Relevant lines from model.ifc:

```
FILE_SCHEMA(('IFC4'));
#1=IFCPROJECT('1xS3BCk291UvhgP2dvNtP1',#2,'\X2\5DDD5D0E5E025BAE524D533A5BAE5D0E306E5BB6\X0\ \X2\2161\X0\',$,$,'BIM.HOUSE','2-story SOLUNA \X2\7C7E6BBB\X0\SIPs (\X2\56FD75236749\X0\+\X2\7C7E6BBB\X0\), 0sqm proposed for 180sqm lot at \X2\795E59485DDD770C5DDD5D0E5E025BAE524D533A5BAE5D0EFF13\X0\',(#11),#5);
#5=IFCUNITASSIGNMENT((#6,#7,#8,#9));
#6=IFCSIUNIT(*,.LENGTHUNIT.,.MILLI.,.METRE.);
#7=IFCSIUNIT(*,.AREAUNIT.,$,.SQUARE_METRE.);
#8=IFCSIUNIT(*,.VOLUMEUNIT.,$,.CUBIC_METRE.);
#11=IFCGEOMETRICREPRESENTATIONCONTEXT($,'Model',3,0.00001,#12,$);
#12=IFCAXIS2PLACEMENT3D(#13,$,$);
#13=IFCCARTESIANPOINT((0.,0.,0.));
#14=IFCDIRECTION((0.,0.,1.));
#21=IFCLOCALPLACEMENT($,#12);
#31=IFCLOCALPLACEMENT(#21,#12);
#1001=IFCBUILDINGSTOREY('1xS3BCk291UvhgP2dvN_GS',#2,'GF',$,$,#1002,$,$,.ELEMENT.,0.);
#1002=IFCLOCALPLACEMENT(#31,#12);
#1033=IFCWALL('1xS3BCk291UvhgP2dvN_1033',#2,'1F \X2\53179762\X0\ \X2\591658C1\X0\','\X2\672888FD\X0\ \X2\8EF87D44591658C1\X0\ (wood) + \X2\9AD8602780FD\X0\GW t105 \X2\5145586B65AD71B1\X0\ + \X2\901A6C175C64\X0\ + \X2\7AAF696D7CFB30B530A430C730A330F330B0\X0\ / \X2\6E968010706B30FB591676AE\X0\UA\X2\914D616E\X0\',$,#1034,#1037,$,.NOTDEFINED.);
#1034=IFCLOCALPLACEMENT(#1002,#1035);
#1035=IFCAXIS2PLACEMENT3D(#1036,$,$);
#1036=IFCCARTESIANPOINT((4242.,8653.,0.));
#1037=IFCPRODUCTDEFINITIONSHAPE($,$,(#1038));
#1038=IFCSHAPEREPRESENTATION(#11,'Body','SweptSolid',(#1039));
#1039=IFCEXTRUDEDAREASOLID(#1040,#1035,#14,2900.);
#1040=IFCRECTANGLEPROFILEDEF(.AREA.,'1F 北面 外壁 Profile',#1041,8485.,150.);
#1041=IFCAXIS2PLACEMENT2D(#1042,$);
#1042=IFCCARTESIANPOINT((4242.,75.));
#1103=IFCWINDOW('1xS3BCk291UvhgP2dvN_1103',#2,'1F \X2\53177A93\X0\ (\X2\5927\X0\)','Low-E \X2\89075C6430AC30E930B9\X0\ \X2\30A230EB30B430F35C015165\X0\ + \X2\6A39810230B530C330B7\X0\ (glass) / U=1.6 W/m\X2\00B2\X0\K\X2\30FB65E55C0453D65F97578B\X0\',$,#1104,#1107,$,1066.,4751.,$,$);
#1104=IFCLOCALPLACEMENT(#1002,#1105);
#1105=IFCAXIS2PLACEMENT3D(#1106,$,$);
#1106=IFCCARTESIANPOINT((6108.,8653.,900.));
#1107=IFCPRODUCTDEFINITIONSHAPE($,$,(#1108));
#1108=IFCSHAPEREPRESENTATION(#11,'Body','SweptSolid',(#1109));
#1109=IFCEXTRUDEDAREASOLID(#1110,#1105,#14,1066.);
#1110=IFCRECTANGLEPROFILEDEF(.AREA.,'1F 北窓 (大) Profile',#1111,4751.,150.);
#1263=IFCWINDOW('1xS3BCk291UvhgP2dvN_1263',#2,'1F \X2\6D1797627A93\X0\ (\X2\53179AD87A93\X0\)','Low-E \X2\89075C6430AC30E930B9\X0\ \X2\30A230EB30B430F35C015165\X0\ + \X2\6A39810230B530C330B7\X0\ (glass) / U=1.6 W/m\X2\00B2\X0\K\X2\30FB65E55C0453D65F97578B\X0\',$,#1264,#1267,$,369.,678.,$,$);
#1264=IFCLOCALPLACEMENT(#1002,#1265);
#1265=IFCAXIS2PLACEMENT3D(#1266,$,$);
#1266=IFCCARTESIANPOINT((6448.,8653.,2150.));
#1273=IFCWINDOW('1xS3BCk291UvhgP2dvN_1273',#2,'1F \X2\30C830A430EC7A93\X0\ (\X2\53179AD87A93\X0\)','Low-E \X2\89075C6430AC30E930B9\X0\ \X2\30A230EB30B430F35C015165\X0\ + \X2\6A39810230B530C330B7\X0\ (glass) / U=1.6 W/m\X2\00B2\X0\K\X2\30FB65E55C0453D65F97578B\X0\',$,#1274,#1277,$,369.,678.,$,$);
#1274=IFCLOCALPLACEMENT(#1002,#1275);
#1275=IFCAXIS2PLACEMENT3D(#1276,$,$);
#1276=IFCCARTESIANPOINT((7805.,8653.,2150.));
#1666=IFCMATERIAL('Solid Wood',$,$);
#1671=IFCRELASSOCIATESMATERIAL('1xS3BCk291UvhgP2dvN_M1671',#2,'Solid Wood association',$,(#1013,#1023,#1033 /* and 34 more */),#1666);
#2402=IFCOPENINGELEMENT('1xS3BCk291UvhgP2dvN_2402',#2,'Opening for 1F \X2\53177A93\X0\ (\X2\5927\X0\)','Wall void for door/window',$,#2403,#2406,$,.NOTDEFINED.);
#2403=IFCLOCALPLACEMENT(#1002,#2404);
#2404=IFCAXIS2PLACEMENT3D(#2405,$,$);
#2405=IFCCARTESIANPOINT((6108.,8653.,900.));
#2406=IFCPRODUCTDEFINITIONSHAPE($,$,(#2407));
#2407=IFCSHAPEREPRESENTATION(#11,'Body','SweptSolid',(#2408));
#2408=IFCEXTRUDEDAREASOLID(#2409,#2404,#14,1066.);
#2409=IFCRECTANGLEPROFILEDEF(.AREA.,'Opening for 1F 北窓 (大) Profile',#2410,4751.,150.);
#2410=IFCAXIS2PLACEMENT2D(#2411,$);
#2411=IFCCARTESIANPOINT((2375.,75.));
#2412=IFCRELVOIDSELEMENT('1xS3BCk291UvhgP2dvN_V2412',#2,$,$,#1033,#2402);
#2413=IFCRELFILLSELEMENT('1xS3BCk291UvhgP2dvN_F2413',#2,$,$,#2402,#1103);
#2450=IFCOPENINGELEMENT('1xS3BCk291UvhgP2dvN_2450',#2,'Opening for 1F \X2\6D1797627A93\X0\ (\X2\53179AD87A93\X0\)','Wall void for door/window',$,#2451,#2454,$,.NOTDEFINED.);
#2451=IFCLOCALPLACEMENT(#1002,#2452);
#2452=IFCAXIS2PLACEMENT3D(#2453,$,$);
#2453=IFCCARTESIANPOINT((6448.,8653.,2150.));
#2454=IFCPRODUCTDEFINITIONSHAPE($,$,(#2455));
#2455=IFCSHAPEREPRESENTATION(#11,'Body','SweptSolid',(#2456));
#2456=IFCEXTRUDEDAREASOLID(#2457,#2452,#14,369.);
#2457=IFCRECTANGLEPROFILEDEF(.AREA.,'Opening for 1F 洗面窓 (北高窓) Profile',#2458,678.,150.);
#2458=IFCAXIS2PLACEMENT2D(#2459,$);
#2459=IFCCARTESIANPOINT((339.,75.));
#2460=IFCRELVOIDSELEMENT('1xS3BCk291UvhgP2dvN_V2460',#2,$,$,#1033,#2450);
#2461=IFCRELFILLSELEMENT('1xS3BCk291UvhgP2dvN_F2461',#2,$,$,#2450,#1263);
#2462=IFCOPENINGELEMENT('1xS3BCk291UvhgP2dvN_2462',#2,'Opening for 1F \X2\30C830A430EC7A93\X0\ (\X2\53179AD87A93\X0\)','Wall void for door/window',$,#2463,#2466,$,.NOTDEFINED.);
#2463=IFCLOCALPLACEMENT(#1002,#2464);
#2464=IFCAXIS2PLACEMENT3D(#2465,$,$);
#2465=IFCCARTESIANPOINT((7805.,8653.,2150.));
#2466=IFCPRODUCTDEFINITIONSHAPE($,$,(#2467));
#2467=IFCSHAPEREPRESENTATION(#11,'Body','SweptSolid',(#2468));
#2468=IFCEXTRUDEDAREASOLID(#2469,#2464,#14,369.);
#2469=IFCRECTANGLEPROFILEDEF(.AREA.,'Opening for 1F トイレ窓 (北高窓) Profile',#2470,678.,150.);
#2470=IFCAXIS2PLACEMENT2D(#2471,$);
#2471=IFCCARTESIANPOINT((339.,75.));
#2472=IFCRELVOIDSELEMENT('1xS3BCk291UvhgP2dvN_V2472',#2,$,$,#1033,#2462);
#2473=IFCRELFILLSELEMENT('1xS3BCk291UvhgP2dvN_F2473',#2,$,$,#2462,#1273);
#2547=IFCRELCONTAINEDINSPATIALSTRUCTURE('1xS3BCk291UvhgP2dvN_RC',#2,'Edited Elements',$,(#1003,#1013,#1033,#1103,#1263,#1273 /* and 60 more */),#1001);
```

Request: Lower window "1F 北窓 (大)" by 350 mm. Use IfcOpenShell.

```python
import numpy as np
import ifcopenshell
import ifcopenshell.api.geometry
import ifcopenshell.util.placement
import ifcopenshell.util.unit

model = ifcopenshell.open("model.ifc")
unit_scale = ifcopenshell.util.unit.calculate_unit_scale(model)

window = model.by_id(1103)
opening = window.FillsVoids[0].RelatingOpeningElement
dz = -0.35 / unit_scale

shift = np.array([0.0, 0.0, dz])
# The window is not placed relative to its opening, so move both.
for product in (opening, window):
    matrix = ifcopenshell.util.placement.get_local_placement(product.ObjectPlacement)
    matrix[:3, 3] += shift
    ifcopenshell.api.geometry.edit_object_placement(model, product=product, matrix=matrix, is_si=False)

print(f"moved by {dz * unit_scale:+.3f} m")

model.write("model-out.ifc")
```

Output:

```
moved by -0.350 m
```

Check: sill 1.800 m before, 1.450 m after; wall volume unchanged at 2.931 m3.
